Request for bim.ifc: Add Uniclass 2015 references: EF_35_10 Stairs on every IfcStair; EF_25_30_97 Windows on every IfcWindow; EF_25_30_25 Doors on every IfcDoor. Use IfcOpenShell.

First a look at what the model holds.

```python
import ifcopenshell

model = ifcopenshell.open("bim.ifc")
print(model.schema)
print("classifications:", [c.Name for c in model.by_type("IfcClassification")])
for ifc_class in ("IfcDoor", "IfcRoof", "IfcStair", "IfcWall", "IfcWindow"):
    print(ifc_class, len(model.by_type(ifc_class)))
```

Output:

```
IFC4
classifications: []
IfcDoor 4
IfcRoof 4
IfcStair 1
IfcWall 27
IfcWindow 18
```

```python
import ifcopenshell
import ifcopenshell.api.classification

model = ifcopenshell.open("bim.ifc")

system = ifcopenshell.api.classification.add_classification(model, classification="Uniclass 2015")

codes = {
    "IfcStair": ("EF_35_10", "Stairs"),
    "IfcWindow": ("EF_25_30_97", "Windows"),
    "IfcDoor": ("EF_25_30_25", "Doors"),
}
for ifc_class, (code, name) in codes.items():
    products = model.by_type(ifc_class)
    ifcopenshell.api.classification.add_reference(
        model, products=products, classification=system, identification=code, name=name
    )
    print(code, len(products))

model.write("bim-out.ifc")
```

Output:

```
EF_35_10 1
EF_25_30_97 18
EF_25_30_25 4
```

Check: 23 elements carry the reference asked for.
